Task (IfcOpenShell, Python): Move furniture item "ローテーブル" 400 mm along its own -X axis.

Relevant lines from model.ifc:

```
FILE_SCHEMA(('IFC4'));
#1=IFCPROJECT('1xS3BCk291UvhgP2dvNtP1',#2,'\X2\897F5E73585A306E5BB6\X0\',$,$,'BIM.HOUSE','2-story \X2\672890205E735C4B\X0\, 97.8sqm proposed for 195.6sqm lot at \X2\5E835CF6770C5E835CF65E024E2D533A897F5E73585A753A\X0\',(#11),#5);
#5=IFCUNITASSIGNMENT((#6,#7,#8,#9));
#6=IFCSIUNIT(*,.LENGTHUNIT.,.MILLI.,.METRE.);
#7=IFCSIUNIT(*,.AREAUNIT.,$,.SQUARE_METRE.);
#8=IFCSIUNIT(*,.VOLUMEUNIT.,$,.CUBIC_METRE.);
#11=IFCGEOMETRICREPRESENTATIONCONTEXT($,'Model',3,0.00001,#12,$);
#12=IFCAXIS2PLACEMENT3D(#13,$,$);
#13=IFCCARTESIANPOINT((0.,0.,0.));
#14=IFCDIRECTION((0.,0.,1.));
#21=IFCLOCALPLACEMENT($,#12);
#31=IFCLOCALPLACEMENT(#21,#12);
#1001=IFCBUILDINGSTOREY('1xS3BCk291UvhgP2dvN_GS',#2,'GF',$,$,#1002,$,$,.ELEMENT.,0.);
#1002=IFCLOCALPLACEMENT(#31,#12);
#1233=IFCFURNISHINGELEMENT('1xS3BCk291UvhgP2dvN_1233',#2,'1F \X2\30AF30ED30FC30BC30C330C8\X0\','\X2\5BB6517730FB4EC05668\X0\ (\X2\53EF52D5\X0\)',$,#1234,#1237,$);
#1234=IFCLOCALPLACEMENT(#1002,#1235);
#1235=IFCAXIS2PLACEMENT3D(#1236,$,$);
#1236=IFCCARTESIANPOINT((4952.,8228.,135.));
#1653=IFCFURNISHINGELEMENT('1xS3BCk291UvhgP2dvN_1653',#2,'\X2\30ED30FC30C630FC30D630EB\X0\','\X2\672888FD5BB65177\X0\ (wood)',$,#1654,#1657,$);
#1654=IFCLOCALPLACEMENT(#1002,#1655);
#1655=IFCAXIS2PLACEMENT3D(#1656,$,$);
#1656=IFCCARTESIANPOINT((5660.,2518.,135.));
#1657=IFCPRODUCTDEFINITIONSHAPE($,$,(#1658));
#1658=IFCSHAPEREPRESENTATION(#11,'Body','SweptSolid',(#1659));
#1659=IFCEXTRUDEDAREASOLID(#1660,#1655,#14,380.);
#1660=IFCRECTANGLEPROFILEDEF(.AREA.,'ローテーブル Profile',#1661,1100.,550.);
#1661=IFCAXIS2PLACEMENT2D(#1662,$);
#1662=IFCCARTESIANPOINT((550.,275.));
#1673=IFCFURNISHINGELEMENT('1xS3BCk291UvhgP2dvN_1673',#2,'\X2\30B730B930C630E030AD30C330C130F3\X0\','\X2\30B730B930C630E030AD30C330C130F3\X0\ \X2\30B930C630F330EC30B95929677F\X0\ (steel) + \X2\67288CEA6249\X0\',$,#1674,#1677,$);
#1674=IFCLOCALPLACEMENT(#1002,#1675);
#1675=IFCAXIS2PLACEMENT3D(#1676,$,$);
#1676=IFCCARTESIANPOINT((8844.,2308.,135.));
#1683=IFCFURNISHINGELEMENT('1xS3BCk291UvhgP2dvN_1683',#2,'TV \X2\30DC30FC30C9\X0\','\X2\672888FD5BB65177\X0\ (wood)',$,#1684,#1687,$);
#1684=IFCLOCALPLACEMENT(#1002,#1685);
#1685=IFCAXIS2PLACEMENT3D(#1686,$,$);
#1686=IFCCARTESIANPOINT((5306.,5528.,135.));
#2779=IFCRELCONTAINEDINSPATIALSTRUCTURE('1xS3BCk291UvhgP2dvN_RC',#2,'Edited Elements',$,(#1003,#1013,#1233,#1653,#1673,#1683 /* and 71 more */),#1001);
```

```python
import ifcopenshell
import ifcopenshell.api.geometry
import ifcopenshell.util.placement
import ifcopenshell.util.unit

model = ifcopenshell.open("model.ifc")
unit_scale = ifcopenshell.util.unit.calculate_unit_scale(model)

item = model.by_id(1653)
matrix = ifcopenshell.util.placement.get_local_placement(item.ObjectPlacement)
matrix[:3, 3] -= matrix[:3, 0] * 0.4 / unit_scale
ifcopenshell.api.geometry.edit_object_placement(model, product=item, matrix=matrix, is_si=False)

print(ifcopenshell.util.placement.get_local_placement(item.ObjectPlacement).round(3) + 0.0)

model.write("model_edited.ifc")
```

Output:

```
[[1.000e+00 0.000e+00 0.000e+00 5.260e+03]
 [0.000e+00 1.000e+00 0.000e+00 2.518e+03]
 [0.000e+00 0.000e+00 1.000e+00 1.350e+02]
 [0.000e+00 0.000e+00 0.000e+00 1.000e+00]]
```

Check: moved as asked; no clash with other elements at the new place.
